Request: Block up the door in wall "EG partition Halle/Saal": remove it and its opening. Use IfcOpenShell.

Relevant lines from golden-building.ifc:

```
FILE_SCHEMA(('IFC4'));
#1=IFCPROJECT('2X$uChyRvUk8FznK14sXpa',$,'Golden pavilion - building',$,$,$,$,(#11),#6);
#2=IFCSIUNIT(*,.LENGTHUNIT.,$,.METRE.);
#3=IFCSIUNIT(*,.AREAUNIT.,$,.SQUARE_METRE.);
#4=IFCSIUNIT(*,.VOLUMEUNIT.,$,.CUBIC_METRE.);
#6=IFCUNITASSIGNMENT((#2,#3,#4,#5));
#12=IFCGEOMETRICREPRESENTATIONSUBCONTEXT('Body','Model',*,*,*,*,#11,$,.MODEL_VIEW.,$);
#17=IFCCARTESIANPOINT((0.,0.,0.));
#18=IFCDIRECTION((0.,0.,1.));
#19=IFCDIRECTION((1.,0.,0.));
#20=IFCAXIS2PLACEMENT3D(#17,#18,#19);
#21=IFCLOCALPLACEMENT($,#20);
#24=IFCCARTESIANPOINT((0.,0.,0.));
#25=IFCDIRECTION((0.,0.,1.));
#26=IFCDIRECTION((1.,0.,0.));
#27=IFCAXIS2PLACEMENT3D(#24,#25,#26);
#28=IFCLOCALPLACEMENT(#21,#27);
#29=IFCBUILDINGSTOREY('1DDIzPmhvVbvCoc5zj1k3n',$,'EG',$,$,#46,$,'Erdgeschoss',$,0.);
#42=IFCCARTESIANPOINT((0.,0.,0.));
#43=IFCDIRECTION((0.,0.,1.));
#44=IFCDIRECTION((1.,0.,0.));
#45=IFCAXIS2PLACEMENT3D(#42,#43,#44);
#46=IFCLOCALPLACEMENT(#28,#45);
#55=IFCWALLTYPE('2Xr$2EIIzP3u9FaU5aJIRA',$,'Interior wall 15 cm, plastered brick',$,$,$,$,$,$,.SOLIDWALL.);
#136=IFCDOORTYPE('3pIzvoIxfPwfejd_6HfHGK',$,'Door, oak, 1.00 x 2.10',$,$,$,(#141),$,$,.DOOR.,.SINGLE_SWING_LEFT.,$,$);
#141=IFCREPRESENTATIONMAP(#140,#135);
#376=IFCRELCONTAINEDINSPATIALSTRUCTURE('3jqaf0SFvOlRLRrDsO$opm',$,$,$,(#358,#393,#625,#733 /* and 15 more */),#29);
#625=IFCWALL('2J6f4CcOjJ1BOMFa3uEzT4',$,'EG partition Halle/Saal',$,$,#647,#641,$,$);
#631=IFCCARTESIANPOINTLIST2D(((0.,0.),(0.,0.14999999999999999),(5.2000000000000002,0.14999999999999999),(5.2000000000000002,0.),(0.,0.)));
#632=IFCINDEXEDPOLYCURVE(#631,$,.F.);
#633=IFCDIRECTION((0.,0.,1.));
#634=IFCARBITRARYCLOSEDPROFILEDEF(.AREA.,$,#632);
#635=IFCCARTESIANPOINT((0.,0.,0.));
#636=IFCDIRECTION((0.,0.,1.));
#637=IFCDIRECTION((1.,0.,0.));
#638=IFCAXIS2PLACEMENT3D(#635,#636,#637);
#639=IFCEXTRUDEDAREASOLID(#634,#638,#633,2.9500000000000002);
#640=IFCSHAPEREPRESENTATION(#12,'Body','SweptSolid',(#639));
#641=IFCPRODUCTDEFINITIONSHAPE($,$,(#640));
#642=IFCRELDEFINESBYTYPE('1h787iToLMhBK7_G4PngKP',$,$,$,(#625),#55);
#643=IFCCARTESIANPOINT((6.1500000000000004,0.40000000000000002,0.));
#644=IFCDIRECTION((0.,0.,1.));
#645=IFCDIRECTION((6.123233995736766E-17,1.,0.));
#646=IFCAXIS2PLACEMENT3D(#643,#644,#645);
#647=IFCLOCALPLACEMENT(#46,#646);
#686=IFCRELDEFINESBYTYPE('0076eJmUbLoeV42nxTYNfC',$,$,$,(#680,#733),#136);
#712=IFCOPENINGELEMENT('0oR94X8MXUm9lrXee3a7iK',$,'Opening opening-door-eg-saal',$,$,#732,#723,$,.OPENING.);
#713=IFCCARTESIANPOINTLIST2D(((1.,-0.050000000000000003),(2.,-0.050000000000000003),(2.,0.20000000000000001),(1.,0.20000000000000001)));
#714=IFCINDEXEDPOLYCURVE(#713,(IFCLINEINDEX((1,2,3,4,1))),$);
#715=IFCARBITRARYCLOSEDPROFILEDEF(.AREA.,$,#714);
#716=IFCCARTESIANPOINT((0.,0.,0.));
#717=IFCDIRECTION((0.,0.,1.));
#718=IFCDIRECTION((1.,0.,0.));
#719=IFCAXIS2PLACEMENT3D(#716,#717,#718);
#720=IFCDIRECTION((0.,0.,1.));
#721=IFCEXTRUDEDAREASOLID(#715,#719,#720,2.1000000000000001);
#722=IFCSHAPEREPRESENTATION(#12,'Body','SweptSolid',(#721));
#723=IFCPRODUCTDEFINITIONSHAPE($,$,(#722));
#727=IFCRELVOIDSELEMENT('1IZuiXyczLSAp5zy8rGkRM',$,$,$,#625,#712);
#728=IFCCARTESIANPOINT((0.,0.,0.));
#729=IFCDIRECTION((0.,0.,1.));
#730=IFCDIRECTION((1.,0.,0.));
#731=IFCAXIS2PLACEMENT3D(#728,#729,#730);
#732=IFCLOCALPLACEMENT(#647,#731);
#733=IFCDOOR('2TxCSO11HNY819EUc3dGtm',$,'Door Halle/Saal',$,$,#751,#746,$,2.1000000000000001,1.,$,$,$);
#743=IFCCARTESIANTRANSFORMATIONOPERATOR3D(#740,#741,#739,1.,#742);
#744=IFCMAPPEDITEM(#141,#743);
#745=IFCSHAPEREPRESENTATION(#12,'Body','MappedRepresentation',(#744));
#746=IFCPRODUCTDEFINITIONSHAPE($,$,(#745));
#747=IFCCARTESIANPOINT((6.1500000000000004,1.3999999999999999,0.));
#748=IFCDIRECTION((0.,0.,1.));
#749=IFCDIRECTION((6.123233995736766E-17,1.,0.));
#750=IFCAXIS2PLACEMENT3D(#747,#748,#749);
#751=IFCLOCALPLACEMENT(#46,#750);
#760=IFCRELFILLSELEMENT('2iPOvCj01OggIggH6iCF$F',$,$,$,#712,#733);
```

```python
import ifcopenshell
import ifcopenshell.api.feature
import ifcopenshell.api.root
import ifcopenshell.geom
import ifcopenshell.util.shape

model = ifcopenshell.open("golden-building.ifc")
settings = ifcopenshell.geom.settings()


def volume(element):
    """Net volume in cubic metres, openings subtracted."""
    shape = ifcopenshell.geom.create_shape(settings, element)
    return ifcopenshell.util.shape.get_volume(shape.geometry)


door = model.by_guid("2TxCSO11HNY819EUc3dGtm")
opening = door.FillsVoids[0].RelatingOpeningElement
wall = opening.VoidsElements[0].RelatingBuildingElement
before = volume(wall)

ifcopenshell.api.root.remove_product(model, product=door)
ifcopenshell.api.feature.remove_feature(model, feature=opening)

after = volume(wall)

print(f"wall volume {before:.3f} -> {after:.3f} m3")

model.write("golden-building-out.ifc")
```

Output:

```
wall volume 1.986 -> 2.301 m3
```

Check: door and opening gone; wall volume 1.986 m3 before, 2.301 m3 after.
